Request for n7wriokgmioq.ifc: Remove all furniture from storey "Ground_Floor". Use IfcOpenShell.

First a look at what the model holds.

```python
import ifcopenshell
import ifcopenshell.util.element

model = ifcopenshell.open("n7wriokgmioq.ifc")
print(model.schema)
storey = next(s for s in model.by_type("IfcBuildingStorey") if s.Name == "Ground_Floor")
furniture = [e for e in ifcopenshell.util.element.get_decomposition(storey) if e.is_a("IfcFurnishingElement")]
seen = {}
for e in furniture:
    element_type = ifcopenshell.util.element.get_type(e)
    name = element_type.Name if element_type not in (None, e) else None
    seen[name] = seen.get(name, 0) + 1
for name, count in sorted(seen.items(), key=str):
    print(count, "x", name)
```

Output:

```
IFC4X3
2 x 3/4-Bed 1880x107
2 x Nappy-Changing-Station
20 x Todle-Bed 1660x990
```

```python
import ifcopenshell
import ifcopenshell.api.root
import ifcopenshell.util.element

model = ifcopenshell.open("n7wriokgmioq.ifc")

storey = next(s for s in model.by_type("IfcBuildingStorey") if s.Name == "Ground_Floor")
furniture = [e for e in ifcopenshell.util.element.get_decomposition(storey) if e.is_a("IfcFurnishingElement")]

for e in furniture:
    ifcopenshell.api.root.remove_product(model, product=e)
print(len(furniture), "removed")

model.write("n7wriokgmioq_v2.ifc")
```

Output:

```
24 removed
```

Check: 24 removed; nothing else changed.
